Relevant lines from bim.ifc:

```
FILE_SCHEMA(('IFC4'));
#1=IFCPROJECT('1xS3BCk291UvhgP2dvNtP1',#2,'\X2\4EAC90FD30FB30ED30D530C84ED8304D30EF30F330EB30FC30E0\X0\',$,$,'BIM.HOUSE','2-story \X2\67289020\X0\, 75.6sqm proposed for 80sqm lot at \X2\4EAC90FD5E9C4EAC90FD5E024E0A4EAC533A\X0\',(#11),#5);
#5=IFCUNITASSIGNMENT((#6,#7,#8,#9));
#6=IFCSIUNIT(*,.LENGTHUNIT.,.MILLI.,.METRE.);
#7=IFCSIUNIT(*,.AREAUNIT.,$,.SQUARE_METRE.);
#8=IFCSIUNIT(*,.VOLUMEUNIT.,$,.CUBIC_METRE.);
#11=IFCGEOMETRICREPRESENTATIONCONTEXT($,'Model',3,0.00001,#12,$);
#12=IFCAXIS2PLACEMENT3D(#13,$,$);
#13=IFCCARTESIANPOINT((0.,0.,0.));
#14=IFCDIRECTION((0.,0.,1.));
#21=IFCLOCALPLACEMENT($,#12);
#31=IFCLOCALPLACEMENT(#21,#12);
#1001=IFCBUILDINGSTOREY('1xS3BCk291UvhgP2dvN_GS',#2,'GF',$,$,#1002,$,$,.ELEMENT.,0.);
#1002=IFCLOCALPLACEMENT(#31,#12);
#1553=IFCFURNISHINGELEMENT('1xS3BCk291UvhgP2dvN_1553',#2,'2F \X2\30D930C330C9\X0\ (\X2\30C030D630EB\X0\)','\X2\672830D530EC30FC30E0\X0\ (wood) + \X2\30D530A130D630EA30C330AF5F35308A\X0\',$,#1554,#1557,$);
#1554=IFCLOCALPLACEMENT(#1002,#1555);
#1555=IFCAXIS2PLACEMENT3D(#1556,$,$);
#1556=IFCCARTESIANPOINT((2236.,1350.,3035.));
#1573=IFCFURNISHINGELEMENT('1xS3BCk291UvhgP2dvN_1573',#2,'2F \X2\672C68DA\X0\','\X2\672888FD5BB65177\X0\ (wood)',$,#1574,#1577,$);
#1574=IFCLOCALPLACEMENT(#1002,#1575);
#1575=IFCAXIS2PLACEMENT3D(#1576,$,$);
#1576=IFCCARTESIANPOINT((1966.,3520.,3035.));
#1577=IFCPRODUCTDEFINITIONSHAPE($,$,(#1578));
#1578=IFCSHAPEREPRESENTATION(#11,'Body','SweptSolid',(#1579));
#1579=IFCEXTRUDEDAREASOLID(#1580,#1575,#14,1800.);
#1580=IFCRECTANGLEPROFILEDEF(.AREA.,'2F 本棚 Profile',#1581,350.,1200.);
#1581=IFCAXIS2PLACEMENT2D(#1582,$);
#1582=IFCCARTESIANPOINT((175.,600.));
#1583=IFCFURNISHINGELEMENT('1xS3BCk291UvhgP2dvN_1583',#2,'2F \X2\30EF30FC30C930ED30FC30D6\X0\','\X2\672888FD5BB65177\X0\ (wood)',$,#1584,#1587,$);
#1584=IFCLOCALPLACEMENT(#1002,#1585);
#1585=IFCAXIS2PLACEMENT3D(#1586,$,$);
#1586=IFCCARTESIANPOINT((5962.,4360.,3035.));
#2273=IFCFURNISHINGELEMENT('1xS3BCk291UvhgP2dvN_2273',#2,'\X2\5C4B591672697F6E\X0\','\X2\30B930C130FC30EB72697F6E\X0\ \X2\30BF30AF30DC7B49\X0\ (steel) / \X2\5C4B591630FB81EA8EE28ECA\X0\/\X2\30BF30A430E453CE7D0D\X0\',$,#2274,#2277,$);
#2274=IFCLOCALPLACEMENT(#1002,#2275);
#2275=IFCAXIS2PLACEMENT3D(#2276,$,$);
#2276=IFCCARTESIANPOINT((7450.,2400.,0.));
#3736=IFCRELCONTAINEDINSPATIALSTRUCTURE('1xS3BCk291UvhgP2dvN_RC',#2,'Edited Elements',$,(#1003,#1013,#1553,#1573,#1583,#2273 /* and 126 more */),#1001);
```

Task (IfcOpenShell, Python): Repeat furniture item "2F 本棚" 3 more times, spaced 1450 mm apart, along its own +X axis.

```python
import ifcopenshell
import ifcopenshell.api.geometry
import ifcopenshell.api.root
import ifcopenshell.util.element
import ifcopenshell.util.placement
import ifcopenshell.util.unit

model = ifcopenshell.open("bim.ifc")
unit_scale = ifcopenshell.util.unit.calculate_unit_scale(model)


def reuse_history(source, copy):
    """copy_class also copies each property set's owner history, people and application; keep the originals."""
    for rel in copy.IsDefinedBy:
        if rel.is_a("IfcRelDefinesByProperties") and (history := rel.RelatingPropertyDefinition.OwnerHistory):
            rel.RelatingPropertyDefinition.OwnerHistory = source.OwnerHistory
            ifcopenshell.util.element.remove_deep2(model, history)


source = model.by_guid("1xS3BCk291UvhgP2dvN_1573")
base = ifcopenshell.util.placement.get_local_placement(source.ObjectPlacement)
step = base[:3, 0] * 1.45 / unit_scale

for i in range(1, 4):
    copy = ifcopenshell.api.root.copy_class(model, product=source)
    copy.Representation = ifcopenshell.util.element.copy_deep(
        model, source.Representation, exclude=["IfcGeometricRepresentationContext", "IfcRepresentationMap"]
    )
    reuse_history(source, copy)
    matrix = base.copy()
    matrix[:3, 3] += i * step
    print("added at", matrix[:3, 3].round(3) + 0.0)
    ifcopenshell.api.geometry.edit_object_placement(model, product=copy, matrix=matrix, is_si=False)

model.write("bim-out.ifc")
```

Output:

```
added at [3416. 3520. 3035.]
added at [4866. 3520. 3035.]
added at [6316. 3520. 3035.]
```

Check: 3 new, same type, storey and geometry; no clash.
